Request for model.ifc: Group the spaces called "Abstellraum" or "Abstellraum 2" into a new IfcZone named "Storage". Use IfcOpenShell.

First a look at what the model holds.

```python
import ifcopenshell

model = ifcopenshell.open("model.ifc")
print(model.schema)
seen = {}
for space in model.by_type("IfcSpace"):
    seen[space.Name] = seen.get(space.Name, 0) + 1
for name, count in sorted(seen.items(), key=str):
    print(count, "x", name)
print("zones:", [z.Name for z in model.by_type("IfcZone")][:20])
```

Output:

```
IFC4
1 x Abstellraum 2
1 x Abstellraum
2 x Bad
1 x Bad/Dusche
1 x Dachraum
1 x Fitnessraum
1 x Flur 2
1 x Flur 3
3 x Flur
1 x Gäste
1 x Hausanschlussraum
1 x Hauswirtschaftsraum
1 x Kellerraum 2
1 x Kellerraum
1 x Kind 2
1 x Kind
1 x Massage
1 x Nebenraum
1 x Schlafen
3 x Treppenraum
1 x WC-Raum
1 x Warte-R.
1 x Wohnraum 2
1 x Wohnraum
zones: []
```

```python
import ifcopenshell
import ifcopenshell.api.group
import ifcopenshell.api.root

model = ifcopenshell.open("model.ifc")

names = {"Abstellraum", "Abstellraum 2"}
spaces = [s for s in model.by_type("IfcSpace") if s.Name in names]

zone = ifcopenshell.api.root.create_entity(model, ifc_class="IfcZone", name="Storage")
ifcopenshell.api.group.assign_group(model, products=spaces, group=zone)
print(len(spaces), "spaces in", zone.Name)

model.write("model_edited.ifc")
```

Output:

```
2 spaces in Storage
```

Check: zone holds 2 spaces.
